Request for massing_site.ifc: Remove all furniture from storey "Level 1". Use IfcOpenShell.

First a look at what the model holds.

```python
import ifcopenshell
import ifcopenshell.util.element

model = ifcopenshell.open("massing_site.ifc")
print(model.schema)
storey = next(s for s in model.by_type("IfcBuildingStorey") if s.Name == "Level 1")
furniture = [e for e in ifcopenshell.util.element.get_decomposition(storey) if e.is_a("IfcFurnishingElement")]
seen = {}
for e in furniture:
    element_type = ifcopenshell.util.element.get_type(e)
    name = element_type.Name if element_type not in (None, e) else None
    seen[name] = seen.get(name, 0) + 1
for name, count in sorted(seen.items(), key=str):
    print(count, "x", name)
```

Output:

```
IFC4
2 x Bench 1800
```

```python
import ifcopenshell
import ifcopenshell.api.root
import ifcopenshell.util.element

model = ifcopenshell.open("massing_site.ifc")

storey = next(s for s in model.by_type("IfcBuildingStorey") if s.Name == "Level 1")
furniture = [e for e in ifcopenshell.util.element.get_decomposition(storey) if e.is_a("IfcFurnishingElement")]

for e in furniture:
    ifcopenshell.api.root.remove_product(model, product=e)
print(len(furniture), "removed")

model.write("massing_site_updated.ifc")
```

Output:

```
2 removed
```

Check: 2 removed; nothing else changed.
